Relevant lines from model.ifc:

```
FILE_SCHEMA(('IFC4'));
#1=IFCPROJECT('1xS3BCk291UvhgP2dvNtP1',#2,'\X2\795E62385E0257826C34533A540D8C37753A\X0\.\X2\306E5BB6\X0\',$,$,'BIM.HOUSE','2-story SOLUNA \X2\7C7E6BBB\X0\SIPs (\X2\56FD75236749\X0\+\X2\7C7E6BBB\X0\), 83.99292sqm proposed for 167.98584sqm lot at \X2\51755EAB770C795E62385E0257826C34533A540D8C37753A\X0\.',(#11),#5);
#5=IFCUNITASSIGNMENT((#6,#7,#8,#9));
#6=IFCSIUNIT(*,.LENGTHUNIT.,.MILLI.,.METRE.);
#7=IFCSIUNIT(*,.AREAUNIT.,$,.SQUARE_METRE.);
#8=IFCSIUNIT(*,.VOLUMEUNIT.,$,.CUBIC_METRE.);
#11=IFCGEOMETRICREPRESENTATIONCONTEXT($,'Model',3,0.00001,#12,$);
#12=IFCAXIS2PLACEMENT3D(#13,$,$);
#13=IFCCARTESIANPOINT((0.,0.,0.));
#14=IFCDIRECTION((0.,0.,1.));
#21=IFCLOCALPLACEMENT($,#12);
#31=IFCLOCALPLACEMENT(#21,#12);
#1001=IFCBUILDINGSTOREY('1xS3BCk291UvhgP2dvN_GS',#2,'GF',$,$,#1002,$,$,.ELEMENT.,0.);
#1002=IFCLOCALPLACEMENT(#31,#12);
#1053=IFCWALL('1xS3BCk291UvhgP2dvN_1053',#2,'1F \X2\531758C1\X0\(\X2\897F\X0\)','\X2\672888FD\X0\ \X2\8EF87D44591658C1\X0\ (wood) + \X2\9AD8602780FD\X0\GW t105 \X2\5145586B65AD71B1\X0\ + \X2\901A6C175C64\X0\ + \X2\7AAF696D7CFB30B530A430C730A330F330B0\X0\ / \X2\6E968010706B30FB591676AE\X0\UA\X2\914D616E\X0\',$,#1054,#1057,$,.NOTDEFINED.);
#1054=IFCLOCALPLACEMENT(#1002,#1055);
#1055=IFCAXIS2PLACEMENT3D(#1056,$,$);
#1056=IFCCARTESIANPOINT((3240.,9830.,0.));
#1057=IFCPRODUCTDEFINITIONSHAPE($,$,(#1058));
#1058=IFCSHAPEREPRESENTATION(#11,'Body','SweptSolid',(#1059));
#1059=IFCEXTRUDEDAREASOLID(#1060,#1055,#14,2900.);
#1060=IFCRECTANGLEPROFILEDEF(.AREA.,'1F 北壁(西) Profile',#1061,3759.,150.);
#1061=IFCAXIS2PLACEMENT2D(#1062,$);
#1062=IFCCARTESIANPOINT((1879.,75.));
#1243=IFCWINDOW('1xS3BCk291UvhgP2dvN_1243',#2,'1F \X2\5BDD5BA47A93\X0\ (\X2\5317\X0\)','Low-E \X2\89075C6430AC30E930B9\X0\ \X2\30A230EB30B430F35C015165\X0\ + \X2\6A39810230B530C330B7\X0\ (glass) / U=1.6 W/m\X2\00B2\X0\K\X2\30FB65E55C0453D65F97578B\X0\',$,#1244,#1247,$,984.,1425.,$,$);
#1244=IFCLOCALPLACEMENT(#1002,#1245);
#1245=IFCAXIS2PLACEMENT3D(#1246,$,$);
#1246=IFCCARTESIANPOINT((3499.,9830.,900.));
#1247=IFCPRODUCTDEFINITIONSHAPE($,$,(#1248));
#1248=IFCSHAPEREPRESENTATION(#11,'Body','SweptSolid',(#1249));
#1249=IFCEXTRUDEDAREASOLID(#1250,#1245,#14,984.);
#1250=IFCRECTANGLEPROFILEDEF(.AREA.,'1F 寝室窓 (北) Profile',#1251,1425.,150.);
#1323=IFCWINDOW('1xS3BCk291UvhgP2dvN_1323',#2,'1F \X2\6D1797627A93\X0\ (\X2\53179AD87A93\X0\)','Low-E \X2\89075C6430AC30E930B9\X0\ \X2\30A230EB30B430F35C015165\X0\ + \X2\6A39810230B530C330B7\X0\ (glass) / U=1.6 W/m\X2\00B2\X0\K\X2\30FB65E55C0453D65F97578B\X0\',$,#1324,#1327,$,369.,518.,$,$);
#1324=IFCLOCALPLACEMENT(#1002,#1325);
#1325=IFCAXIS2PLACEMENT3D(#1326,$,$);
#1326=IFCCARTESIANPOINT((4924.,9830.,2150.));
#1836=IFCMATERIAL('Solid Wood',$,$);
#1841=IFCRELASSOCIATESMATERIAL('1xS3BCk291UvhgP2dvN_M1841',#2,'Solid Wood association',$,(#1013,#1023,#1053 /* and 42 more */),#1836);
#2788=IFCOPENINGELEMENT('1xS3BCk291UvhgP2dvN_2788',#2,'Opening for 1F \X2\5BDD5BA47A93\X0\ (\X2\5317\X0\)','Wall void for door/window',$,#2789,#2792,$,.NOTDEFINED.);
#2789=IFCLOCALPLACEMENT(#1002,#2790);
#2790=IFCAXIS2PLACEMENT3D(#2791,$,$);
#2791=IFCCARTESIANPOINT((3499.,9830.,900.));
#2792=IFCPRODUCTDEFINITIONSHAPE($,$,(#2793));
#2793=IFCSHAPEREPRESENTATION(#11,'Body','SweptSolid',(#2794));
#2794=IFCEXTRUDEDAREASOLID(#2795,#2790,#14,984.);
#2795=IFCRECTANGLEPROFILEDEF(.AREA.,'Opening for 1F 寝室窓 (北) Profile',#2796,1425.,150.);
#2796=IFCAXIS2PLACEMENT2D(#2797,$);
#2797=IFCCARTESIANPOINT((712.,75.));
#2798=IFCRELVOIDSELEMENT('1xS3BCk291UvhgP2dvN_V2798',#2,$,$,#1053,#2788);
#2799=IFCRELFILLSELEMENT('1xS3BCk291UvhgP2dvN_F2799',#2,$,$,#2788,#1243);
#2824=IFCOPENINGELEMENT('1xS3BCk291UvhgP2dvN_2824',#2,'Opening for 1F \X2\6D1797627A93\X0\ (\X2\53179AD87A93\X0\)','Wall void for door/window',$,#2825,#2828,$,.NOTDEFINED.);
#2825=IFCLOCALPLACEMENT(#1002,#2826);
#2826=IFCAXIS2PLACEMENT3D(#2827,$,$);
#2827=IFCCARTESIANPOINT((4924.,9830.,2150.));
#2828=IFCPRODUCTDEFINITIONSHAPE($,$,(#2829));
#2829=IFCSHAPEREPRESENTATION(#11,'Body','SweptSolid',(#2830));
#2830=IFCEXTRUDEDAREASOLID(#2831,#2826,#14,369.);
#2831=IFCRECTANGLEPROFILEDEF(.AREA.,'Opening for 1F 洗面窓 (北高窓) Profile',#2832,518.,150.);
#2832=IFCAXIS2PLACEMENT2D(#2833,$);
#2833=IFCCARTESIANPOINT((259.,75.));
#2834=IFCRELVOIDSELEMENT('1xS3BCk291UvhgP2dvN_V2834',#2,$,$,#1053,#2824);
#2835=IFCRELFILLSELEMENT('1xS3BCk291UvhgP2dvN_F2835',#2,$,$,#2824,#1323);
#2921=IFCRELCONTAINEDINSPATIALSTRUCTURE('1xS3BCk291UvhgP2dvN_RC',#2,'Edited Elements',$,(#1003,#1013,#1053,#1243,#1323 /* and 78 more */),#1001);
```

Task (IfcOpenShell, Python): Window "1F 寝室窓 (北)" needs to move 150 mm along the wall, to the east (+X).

```python
import ifcopenshell
import ifcopenshell.api.geometry
import ifcopenshell.util.placement

model = ifcopenshell.open("model.ifc")

window = model.by_guid("1xS3BCk291UvhgP2dvN_1243")
opening = window.FillsVoids[0].RelatingOpeningElement
wall = opening.VoidsElements[0].RelatingBuildingElement

wall_matrix = ifcopenshell.util.placement.get_local_placement(wall.ObjectPlacement)
shift = wall_matrix[:3, 0] * 150.0
before = ifcopenshell.util.placement.get_local_placement(window.ObjectPlacement)[:3, 3].copy()

# The window is not placed relative to its opening, so move both.
for product in (opening, window):
    matrix = ifcopenshell.util.placement.get_local_placement(product.ObjectPlacement)
    matrix[:3, 3] += shift
    ifcopenshell.api.geometry.edit_object_placement(model, product=product, matrix=matrix, is_si=False)

after = ifcopenshell.util.placement.get_local_placement(window.ObjectPlacement)[:3, 3]
print("window moved by", (after - before).round(3) + 0.0)

model.write("model_updated.ifc")
```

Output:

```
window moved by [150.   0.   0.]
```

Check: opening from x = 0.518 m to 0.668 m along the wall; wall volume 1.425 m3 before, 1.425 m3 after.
